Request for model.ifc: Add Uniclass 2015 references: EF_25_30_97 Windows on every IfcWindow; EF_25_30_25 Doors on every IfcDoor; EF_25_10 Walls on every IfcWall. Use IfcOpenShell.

First a look at what the model holds.

```python
import ifcopenshell

model = ifcopenshell.open("model.ifc")
print(model.schema)
print("classifications:", [c.Name for c in model.by_type("IfcClassification")])
for ifc_class in ("IfcDoor", "IfcRoof", "IfcStair", "IfcWall", "IfcWindow"):
    print(ifc_class, len(model.by_type(ifc_class)))
```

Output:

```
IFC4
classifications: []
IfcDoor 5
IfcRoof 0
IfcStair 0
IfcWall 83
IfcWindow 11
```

```python
import ifcopenshell
import ifcopenshell.api.classification

model = ifcopenshell.open("model.ifc")

system = ifcopenshell.api.classification.add_classification(model, classification="Uniclass 2015")

codes = {
    "IfcWindow": ("EF_25_30_97", "Windows"),
    "IfcDoor": ("EF_25_30_25", "Doors"),
    "IfcWall": ("EF_25_10", "Walls"),
}
for ifc_class, (code, name) in codes.items():
    products = model.by_type(ifc_class)
    ifcopenshell.api.classification.add_reference(
        model, products=products, classification=system, identification=code, name=name
    )
    print(code, len(products))

model.write("model_updated.ifc")
```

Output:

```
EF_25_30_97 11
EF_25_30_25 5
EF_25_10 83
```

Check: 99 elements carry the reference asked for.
